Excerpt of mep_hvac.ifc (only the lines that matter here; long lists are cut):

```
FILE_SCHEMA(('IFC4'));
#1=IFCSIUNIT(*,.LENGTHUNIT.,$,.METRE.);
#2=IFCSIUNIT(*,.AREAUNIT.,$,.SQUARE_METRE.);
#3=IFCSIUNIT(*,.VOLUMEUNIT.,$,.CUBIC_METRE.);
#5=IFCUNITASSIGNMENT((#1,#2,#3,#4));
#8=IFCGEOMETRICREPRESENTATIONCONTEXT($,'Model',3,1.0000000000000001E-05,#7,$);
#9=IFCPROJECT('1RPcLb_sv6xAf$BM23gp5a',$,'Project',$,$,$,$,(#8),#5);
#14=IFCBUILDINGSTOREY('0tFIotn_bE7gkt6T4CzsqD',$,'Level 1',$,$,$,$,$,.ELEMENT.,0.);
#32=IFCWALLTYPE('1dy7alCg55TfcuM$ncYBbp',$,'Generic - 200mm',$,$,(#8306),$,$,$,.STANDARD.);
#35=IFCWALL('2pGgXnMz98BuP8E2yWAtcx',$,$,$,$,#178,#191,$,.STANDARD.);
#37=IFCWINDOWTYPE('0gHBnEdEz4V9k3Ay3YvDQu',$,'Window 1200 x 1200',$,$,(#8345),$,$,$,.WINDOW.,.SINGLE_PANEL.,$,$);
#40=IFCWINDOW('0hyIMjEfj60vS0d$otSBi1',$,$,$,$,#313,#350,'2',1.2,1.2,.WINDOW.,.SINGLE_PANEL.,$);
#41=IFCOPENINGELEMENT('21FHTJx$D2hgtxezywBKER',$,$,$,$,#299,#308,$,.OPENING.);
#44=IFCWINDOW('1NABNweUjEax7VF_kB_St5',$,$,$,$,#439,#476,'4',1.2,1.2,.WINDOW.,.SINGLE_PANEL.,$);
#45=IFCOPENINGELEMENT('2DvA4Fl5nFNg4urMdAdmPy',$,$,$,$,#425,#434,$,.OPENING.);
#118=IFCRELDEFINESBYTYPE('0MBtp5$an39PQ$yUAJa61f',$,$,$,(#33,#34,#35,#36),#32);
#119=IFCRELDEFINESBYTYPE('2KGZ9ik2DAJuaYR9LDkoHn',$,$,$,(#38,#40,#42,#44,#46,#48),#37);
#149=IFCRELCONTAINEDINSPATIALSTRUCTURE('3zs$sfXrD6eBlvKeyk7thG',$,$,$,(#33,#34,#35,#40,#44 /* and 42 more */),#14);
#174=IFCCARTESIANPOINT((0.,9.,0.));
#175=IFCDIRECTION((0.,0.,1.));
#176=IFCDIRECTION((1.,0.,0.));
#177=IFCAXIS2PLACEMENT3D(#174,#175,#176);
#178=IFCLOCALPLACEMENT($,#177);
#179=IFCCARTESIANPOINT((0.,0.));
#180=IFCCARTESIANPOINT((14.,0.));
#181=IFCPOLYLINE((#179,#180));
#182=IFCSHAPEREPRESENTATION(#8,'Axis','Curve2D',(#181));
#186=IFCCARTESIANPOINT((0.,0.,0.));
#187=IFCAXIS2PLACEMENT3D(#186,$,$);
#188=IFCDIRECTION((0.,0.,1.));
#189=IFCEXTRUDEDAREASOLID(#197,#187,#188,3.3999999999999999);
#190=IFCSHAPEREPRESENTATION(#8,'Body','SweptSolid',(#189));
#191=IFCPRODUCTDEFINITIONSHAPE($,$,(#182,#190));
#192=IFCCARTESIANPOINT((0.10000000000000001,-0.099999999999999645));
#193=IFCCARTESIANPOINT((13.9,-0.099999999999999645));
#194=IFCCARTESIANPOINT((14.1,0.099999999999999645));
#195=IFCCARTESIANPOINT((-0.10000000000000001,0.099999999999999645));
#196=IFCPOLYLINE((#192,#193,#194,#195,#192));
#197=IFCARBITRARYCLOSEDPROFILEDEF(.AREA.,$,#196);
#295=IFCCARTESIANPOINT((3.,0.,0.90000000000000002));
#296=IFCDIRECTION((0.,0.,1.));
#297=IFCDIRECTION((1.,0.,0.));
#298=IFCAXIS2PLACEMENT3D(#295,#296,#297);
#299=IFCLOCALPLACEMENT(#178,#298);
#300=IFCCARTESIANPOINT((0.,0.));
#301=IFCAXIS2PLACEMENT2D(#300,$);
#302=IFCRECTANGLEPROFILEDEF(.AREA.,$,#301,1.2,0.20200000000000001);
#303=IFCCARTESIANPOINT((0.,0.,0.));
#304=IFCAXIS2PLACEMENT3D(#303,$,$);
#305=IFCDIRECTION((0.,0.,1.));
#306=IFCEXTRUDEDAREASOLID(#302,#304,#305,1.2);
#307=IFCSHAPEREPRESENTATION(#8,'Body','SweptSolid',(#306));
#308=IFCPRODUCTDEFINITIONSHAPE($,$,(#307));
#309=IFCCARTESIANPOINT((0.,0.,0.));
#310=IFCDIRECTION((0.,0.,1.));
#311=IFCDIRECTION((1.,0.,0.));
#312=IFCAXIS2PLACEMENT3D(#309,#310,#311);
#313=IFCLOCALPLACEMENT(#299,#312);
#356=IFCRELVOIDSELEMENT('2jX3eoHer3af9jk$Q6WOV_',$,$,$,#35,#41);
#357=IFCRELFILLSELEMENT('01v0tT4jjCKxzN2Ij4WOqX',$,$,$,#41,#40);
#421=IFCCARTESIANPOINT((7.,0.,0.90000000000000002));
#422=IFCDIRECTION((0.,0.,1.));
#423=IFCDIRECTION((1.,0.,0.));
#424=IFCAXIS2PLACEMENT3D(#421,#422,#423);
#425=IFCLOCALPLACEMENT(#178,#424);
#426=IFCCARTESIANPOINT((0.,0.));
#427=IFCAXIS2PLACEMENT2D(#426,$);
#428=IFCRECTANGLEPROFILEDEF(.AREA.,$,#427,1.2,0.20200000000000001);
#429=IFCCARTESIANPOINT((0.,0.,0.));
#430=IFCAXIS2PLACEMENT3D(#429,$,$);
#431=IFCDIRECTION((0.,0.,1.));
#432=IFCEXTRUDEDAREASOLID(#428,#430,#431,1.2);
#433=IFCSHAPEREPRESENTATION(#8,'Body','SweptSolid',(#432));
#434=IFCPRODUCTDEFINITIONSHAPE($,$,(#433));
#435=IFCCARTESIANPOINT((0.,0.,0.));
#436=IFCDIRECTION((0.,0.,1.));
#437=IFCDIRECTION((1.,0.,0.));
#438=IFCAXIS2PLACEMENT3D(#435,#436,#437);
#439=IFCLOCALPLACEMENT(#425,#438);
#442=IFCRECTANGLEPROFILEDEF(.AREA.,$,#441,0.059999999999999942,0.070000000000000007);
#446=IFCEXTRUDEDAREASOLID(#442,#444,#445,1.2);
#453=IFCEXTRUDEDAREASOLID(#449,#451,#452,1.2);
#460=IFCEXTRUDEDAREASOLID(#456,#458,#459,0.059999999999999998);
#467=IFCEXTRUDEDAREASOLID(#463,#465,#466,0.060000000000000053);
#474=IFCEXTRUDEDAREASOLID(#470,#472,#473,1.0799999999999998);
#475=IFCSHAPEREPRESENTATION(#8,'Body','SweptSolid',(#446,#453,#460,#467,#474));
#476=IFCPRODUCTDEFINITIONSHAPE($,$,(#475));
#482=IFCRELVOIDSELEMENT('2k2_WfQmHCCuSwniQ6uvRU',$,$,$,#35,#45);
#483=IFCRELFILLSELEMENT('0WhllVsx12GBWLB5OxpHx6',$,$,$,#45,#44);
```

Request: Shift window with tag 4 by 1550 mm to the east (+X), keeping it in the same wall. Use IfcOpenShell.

```python
import ifcopenshell
import ifcopenshell.api.geometry
import ifcopenshell.util.placement
import ifcopenshell.util.unit

model = ifcopenshell.open("mep_hvac.ifc")
unit_scale = ifcopenshell.util.unit.calculate_unit_scale(model)

window = model.by_id(44)
opening = window.FillsVoids[0].RelatingOpeningElement
wall = opening.VoidsElements[0].RelatingBuildingElement

wall_matrix = ifcopenshell.util.placement.get_local_placement(wall.ObjectPlacement)
shift = wall_matrix[:3, 0] * 1.55 / unit_scale
before = ifcopenshell.util.placement.get_local_placement(window.ObjectPlacement)[:3, 3].copy()

# The window is placed relative to its opening, so it follows when the opening moves.
matrix = ifcopenshell.util.placement.get_local_placement(opening.ObjectPlacement)
matrix[:3, 3] += shift
ifcopenshell.api.geometry.edit_object_placement(
    model, product=opening, matrix=matrix, is_si=False, should_transform_children=True
)

after = ifcopenshell.util.placement.get_local_placement(window.ObjectPlacement)[:3, 3]
print("window moved by", (after - before).round(3) + 0.0)

model.write("mep_hvac_updated.ifc")
```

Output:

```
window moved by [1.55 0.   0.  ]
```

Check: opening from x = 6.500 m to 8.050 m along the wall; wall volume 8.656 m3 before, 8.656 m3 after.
